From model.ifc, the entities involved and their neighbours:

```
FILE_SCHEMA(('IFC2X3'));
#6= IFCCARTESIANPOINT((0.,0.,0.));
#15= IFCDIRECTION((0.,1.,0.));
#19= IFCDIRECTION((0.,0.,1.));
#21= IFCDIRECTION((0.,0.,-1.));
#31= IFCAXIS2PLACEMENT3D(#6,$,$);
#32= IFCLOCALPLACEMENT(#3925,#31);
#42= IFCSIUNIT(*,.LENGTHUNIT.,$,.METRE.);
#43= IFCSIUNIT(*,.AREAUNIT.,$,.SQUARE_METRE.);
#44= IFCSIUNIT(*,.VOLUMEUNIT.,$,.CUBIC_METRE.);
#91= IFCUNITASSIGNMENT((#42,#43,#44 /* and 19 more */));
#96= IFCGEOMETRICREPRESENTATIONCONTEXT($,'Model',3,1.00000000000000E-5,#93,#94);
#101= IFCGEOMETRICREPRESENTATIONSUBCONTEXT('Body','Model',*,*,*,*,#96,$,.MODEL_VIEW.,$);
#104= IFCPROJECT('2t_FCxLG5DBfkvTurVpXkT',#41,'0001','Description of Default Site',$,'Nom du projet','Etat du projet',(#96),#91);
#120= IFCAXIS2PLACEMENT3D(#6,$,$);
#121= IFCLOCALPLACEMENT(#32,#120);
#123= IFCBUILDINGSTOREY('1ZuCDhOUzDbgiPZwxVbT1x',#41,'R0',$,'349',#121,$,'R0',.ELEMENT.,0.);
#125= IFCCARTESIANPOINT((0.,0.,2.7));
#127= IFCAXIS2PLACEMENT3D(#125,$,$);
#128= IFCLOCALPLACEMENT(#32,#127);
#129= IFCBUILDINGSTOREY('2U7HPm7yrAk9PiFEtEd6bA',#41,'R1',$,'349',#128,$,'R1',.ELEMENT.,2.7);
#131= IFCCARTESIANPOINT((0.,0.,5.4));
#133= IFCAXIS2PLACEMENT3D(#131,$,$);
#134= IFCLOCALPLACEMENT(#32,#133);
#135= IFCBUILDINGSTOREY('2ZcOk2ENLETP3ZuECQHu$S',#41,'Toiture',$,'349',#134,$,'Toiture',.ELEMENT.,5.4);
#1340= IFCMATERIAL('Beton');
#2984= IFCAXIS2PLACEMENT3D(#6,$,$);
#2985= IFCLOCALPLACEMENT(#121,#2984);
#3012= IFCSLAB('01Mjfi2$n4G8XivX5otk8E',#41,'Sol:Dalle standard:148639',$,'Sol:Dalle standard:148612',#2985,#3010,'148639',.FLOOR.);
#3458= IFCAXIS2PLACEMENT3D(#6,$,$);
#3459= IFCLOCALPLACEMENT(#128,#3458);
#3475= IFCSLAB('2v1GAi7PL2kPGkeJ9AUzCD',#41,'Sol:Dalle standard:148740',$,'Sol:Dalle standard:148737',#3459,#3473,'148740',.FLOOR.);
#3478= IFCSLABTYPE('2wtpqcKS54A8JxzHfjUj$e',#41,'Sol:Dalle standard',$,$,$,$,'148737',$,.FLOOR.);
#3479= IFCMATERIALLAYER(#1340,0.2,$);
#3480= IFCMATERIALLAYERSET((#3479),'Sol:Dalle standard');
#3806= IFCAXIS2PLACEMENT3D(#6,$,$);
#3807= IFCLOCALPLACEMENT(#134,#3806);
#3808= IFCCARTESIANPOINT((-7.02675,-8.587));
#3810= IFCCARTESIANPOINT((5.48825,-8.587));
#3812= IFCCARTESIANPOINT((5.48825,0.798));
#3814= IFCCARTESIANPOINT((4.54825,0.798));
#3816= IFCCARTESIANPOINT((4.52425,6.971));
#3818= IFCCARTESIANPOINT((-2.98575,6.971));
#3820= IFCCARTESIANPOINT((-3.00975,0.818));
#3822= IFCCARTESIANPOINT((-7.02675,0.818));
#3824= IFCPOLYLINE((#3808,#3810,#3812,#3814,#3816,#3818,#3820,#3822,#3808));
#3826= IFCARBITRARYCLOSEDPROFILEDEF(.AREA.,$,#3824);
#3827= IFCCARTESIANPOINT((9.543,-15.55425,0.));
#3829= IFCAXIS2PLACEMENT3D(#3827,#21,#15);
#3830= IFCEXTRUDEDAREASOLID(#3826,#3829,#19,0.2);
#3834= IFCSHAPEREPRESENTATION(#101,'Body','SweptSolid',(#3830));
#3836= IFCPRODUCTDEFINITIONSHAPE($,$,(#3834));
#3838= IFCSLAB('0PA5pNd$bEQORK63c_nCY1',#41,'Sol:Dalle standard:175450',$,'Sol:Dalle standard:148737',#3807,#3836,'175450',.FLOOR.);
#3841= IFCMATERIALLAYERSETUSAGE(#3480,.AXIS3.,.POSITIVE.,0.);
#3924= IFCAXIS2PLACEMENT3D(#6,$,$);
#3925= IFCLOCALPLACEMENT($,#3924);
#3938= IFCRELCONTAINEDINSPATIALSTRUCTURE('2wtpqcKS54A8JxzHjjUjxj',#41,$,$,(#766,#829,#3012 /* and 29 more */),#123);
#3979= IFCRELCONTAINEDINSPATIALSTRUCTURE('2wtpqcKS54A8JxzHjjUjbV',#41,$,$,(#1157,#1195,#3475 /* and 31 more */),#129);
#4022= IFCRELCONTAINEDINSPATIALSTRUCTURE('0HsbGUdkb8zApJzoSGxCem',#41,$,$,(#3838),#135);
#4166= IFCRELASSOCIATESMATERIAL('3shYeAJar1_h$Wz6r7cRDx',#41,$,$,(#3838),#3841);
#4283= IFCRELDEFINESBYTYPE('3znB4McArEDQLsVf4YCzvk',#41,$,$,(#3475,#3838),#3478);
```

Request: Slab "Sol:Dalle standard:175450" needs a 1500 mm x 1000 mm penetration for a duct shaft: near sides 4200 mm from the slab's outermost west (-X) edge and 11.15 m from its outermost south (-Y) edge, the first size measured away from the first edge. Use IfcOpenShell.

```python
import numpy as np
import ifcopenshell
import ifcopenshell.api.feature
import ifcopenshell.api.geometry
import ifcopenshell.api.root
import ifcopenshell.geom
import ifcopenshell.util.placement
import ifcopenshell.util.representation
import ifcopenshell.util.shape
import ifcopenshell.util.unit

model = ifcopenshell.open("model.ifc")
unit_scale = ifcopenshell.util.unit.calculate_unit_scale(model)
settings = ifcopenshell.geom.settings()


def volume(element):
    """Net volume in cubic metres, openings subtracted."""
    shape = ifcopenshell.geom.create_shape(settings, element)
    return ifcopenshell.util.shape.get_volume(shape.geometry)


slab = model.by_guid("0PA5pNd$bEQORK63c_nCY1")
before = volume(slab)

# Extent in the slab's own axes, in metres. The edges named are its -X and -Y sides.
slab_shape = ifcopenshell.geom.create_shape(settings, slab)
vertices = ifcopenshell.util.shape.get_vertices(slab_shape.geometry)
x_min, y_min, bottom = vertices.min(axis=0)
top = vertices[:, 2].max()

opening = ifcopenshell.api.root.create_entity(model, ifc_class="IfcOpeningElement", name="Duct shaft opening")
context = ifcopenshell.util.representation.get_context(model, "Model", "Body", "MODEL_VIEW")
width, depth = 1.5, 1
outline = [(0.0, 0.0), (width, 0.0), (width, depth), (0.0, depth), (0.0, 0.0)]
# Overshoot both faces by 50 mm so the cut is clean.
shape = ifcopenshell.api.geometry.add_slab_representation(
    model, context=context, depth=top - bottom + 0.1, polyline=outline
)
ifcopenshell.api.geometry.assign_representation(model, product=opening, representation=shape)

matrix = ifcopenshell.util.placement.get_local_placement(slab.ObjectPlacement)
matrix[:, 3] = matrix @ np.append(np.array([x_min + 4.2, y_min + 11.15, bottom - 0.05]) / unit_scale, 1.0)
ifcopenshell.api.geometry.edit_object_placement(model, product=opening, matrix=matrix, is_si=False)
ifcopenshell.api.feature.add_feature(model, feature=opening, element=slab)

after = volume(slab)

print(f"slab volume {before:.3f} -> {after:.3f} m3")

model.write("model_v2.ifc")
```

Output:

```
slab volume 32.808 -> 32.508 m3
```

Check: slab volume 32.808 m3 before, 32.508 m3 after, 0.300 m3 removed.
